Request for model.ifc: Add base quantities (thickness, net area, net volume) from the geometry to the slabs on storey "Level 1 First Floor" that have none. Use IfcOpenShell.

First a look at what the model holds.

```python
import ifcopenshell
import ifcopenshell.util.element
import ifcopenshell.util.unit

model = ifcopenshell.open("model.ifc")
print(model.schema)
for unit_type in ("LENGTHUNIT", "AREAUNIT", "VOLUMEUNIT"):
    print(unit_type, ifcopenshell.util.unit.calculate_unit_scale(model, unit_type))
storey = next(s for s in model.by_type("IfcBuildingStorey") if s.Name == "Level 1 First Floor")
slabs = [e for e in ifcopenshell.util.element.get_decomposition(storey) if e.is_a("IfcSlab")]
for e in sorted(slabs, key=lambda e: e.id()):
    print(e.id(), e.is_a(), e.Name, list(ifcopenshell.util.element.get_psets(e, qtos_only=True)), sep=" | ")
```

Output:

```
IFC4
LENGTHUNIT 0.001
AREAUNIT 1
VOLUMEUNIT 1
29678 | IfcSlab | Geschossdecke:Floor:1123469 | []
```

```python
import ifcopenshell
import ifcopenshell.api.pset
import ifcopenshell.geom
import ifcopenshell.util.element
import ifcopenshell.util.shape
import ifcopenshell.util.unit

model = ifcopenshell.open("model.ifc")
unit_scale = ifcopenshell.util.unit.calculate_unit_scale(model)
area_scale = ifcopenshell.util.unit.calculate_unit_scale(model, "AREAUNIT")
volume_scale = ifcopenshell.util.unit.calculate_unit_scale(model, "VOLUMEUNIT")
settings = ifcopenshell.geom.settings()

storey = next(s for s in model.by_type("IfcBuildingStorey") if s.Name == "Level 1 First Floor")
slabs = [e for e in ifcopenshell.util.element.get_decomposition(storey) if e.is_a("IfcSlab")]

for e in sorted(slabs, key=lambda e: e.id()):
    if ifcopenshell.util.element.get_psets(e, qtos_only=True, should_inherit=False):
        continue
    # Geometry comes back in metres, in the element's own axes.
    shape = ifcopenshell.geom.create_shape(settings, e)
    values = {
        "Width": ifcopenshell.util.shape.get_z(shape.geometry) / unit_scale,
        "NetArea": ifcopenshell.util.shape.get_footprint_area(shape.geometry) / area_scale,
        "NetVolume": ifcopenshell.util.shape.get_volume(shape.geometry) / volume_scale,
    }
    qto = ifcopenshell.api.pset.add_qto(model, product=e, name="Qto_SlabBaseQuantities")
    ifcopenshell.api.pset.edit_qto(model, qto=qto, properties=values)
    print(e.id(), {k: round(v, 3) for k, v in values.items()})

model.write("model_rev.ifc")
```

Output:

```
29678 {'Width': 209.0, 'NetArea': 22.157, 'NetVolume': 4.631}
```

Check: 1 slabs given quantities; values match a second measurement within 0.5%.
